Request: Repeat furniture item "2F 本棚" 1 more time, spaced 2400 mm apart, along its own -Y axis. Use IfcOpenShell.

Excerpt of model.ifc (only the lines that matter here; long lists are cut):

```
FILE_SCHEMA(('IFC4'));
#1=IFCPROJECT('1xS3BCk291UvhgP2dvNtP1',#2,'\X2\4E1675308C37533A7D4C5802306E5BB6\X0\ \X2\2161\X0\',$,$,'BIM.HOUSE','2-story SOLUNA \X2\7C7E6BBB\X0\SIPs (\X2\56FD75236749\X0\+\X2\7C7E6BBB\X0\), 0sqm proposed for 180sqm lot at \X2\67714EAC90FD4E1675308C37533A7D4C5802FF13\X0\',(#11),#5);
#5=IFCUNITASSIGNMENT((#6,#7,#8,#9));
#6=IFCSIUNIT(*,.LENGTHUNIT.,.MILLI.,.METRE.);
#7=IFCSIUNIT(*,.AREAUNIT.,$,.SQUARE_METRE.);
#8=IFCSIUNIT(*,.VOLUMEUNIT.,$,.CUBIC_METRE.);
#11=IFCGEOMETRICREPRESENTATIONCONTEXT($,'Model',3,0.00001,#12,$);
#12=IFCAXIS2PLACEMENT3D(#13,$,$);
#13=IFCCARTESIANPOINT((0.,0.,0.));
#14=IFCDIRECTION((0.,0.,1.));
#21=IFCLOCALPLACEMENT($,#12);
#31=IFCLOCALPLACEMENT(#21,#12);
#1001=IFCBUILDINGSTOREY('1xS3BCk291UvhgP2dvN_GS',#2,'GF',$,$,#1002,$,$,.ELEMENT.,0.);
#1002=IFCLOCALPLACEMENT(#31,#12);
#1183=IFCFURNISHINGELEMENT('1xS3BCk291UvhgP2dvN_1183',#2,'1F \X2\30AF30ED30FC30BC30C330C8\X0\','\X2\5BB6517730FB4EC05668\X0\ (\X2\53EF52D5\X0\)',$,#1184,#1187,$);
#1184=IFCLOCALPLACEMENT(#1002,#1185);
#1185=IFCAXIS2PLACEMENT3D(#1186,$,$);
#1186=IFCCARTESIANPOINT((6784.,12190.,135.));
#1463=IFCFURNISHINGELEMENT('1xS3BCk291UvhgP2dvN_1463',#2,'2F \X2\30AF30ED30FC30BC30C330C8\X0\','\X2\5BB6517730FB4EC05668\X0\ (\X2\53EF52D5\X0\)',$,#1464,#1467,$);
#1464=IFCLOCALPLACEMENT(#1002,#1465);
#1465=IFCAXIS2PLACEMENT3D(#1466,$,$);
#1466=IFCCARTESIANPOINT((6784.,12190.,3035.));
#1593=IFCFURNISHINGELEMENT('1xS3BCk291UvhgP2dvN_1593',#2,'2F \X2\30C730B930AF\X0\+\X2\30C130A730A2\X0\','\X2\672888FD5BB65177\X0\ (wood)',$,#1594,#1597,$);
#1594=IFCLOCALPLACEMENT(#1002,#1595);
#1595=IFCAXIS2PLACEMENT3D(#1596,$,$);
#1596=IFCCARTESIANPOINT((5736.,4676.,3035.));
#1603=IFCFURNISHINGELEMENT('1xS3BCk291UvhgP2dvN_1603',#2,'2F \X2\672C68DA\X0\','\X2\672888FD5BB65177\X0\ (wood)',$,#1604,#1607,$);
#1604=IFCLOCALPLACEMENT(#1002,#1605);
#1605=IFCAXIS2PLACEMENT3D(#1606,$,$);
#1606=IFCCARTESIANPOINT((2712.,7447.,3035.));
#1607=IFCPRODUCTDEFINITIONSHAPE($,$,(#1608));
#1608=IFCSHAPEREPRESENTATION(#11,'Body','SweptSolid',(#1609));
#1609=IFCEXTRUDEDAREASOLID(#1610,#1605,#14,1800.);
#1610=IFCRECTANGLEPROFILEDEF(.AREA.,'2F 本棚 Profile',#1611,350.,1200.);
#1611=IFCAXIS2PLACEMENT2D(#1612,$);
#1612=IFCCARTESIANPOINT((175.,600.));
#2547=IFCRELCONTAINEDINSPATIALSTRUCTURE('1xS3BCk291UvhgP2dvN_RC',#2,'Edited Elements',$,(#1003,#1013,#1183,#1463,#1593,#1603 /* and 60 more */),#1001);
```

```python
import ifcopenshell
import ifcopenshell.api.geometry
import ifcopenshell.api.root
import ifcopenshell.util.element
import ifcopenshell.util.placement

model = ifcopenshell.open("model.ifc")


def reuse_history(source, copy):
    """copy_class also copies each property set's owner history, people and application; keep the originals."""
    for rel in copy.IsDefinedBy:
        if rel.is_a("IfcRelDefinesByProperties") and (history := rel.RelatingPropertyDefinition.OwnerHistory):
            rel.RelatingPropertyDefinition.OwnerHistory = source.OwnerHistory
            ifcopenshell.util.element.remove_deep2(model, history)


source = model.by_id(1603)
base = ifcopenshell.util.placement.get_local_placement(source.ObjectPlacement)
step = -base[:3, 1] * 2400.0

for i in range(1, 2):
    copy = ifcopenshell.api.root.copy_class(model, product=source)
    copy.Representation = ifcopenshell.util.element.copy_deep(
        model, source.Representation, exclude=["IfcGeometricRepresentationContext", "IfcRepresentationMap"]
    )
    reuse_history(source, copy)
    matrix = base.copy()
    matrix[:3, 3] += i * step
    print("added at", matrix[:3, 3].round(3) + 0.0)
    ifcopenshell.api.geometry.edit_object_placement(model, product=copy, matrix=matrix, is_si=False)

model.write("model_edited.ifc")
```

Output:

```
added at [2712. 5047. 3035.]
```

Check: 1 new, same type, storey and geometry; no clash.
